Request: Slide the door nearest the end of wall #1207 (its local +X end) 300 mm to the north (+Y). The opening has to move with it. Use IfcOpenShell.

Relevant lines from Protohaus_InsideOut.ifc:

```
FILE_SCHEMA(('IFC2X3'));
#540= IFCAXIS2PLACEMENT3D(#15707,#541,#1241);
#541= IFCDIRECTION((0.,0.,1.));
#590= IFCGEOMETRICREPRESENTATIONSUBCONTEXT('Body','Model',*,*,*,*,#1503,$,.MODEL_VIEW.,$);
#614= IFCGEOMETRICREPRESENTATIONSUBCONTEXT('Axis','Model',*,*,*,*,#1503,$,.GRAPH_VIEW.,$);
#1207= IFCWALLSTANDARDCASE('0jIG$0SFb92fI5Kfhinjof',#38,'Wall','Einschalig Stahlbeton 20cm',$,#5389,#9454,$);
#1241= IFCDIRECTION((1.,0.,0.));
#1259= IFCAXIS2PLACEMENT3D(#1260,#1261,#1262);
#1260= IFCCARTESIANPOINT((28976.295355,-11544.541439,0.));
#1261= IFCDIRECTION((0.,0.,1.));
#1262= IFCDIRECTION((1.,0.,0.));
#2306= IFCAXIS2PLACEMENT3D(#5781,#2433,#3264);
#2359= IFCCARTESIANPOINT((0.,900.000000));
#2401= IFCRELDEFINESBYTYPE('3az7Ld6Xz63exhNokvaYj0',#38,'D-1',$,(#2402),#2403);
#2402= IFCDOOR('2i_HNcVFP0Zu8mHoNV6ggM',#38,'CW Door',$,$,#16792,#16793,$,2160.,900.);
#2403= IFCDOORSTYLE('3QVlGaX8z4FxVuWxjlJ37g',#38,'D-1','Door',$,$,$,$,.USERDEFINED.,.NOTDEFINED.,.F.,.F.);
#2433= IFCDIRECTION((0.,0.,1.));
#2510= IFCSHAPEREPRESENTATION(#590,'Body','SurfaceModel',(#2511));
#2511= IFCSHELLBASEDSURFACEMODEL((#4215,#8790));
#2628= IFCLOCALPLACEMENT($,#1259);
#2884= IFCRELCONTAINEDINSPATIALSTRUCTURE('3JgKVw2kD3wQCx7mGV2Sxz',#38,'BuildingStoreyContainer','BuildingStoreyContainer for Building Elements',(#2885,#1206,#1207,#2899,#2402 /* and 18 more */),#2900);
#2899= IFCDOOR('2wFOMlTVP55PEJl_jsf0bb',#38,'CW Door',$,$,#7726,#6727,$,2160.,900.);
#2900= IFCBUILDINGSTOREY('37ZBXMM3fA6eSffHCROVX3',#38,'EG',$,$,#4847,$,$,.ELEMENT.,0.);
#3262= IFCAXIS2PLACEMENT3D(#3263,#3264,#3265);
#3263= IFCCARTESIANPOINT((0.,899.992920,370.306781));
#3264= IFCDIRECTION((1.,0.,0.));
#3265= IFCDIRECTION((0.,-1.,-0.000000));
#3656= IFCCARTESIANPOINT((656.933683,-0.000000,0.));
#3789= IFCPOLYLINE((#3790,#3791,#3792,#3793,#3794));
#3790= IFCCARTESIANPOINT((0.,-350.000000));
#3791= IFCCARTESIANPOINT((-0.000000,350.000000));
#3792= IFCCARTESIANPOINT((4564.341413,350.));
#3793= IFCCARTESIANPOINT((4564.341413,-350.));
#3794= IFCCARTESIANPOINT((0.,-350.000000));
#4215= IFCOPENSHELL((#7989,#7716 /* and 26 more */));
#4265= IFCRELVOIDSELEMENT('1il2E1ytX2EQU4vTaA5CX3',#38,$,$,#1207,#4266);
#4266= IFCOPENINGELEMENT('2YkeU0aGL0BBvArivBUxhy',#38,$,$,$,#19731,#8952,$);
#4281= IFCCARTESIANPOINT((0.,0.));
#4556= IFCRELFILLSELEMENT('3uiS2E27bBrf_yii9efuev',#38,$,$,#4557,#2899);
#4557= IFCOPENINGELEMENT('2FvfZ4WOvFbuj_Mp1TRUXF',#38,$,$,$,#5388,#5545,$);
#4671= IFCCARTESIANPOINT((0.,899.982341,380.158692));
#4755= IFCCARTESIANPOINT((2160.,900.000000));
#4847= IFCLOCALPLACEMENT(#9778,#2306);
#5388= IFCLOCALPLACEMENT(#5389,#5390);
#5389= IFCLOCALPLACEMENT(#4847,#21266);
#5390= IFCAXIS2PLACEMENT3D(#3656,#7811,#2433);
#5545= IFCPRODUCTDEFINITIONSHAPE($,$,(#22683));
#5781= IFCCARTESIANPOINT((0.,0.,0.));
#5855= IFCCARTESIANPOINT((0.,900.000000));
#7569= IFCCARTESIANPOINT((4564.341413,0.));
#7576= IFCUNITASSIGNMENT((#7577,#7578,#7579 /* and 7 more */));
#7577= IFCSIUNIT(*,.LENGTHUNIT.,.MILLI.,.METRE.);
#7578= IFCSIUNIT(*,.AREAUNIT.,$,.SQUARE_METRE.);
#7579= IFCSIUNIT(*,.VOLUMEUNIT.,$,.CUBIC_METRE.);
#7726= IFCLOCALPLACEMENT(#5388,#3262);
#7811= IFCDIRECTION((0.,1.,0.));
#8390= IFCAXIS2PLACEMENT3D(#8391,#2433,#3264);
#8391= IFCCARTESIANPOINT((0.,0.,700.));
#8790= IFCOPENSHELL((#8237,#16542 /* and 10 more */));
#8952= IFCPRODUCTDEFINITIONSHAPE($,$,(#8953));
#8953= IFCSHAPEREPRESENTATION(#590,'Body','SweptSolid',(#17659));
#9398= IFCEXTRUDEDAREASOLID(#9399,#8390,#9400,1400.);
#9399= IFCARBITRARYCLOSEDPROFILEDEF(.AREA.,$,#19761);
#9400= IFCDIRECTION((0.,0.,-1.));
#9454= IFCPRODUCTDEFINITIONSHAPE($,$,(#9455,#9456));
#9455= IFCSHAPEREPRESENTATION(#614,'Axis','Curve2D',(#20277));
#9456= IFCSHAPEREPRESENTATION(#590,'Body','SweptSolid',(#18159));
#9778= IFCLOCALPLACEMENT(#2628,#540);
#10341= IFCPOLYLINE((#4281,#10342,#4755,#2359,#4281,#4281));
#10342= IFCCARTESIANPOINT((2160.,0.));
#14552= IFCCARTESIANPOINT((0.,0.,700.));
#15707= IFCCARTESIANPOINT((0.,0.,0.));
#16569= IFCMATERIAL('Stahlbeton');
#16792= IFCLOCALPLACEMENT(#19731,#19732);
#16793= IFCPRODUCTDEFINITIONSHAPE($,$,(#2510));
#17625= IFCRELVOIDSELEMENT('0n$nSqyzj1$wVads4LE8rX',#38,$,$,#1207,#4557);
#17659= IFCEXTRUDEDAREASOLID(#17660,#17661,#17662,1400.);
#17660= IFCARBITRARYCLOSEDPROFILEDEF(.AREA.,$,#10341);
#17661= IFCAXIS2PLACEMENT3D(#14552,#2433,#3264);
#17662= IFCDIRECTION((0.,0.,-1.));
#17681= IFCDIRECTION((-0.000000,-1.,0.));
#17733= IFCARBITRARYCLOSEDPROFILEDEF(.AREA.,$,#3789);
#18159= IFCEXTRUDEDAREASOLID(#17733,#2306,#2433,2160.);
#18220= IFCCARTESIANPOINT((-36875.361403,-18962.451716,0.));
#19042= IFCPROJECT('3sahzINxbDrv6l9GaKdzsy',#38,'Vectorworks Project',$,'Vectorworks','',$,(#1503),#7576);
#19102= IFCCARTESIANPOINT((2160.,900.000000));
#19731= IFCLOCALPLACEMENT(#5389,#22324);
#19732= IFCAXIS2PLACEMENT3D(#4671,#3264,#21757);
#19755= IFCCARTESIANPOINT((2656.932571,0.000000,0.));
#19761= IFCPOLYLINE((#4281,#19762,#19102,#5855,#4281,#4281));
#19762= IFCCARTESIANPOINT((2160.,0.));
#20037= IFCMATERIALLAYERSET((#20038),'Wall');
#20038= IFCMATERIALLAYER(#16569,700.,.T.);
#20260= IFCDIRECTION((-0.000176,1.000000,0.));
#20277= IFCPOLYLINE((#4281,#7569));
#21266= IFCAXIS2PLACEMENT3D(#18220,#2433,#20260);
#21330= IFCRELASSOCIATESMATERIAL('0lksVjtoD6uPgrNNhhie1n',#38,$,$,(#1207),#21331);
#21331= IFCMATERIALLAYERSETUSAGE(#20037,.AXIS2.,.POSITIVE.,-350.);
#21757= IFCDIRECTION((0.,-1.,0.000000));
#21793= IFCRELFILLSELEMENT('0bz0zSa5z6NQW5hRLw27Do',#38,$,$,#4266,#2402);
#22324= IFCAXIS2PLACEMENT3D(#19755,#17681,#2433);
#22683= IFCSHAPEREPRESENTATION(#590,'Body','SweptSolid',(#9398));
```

```python
import ifcopenshell
import ifcopenshell.api.geometry
import ifcopenshell.util.placement
import ifcopenshell.util.unit

model = ifcopenshell.open("Protohaus_InsideOut.ifc")
unit_scale = ifcopenshell.util.unit.calculate_unit_scale(model)

door = model.by_guid("2i_HNcVFP0Zu8mHoNV6ggM")
opening = door.FillsVoids[0].RelatingOpeningElement
wall = opening.VoidsElements[0].RelatingBuildingElement

wall_matrix = ifcopenshell.util.placement.get_local_placement(wall.ObjectPlacement)
shift = wall_matrix[:3, 0] * 0.3 / unit_scale
before = ifcopenshell.util.placement.get_local_placement(door.ObjectPlacement)[:3, 3].copy()

# The door is placed relative to its opening, so it follows when the opening moves.
matrix = ifcopenshell.util.placement.get_local_placement(opening.ObjectPlacement)
matrix[:3, 3] += shift
ifcopenshell.api.geometry.edit_object_placement(
    model, product=opening, matrix=matrix, is_si=False, should_transform_children=True
)

after = ifcopenshell.util.placement.get_local_placement(door.ObjectPlacement)[:3, 3]
print("door moved by", (after - before).round(3) + 0.0)

model.write("Protohaus_InsideOut_edited.ifc")
```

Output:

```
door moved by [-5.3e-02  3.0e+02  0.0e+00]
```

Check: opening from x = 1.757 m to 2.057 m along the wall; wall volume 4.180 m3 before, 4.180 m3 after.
